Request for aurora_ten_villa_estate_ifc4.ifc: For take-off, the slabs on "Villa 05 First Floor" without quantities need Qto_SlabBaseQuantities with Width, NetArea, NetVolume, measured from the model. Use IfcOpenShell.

First a look at what the model holds.

```python
import ifcopenshell
import ifcopenshell.util.element
import ifcopenshell.util.unit

model = ifcopenshell.open("aurora_ten_villa_estate_ifc4.ifc")
print(model.schema)
for unit_type in ("LENGTHUNIT", "AREAUNIT", "VOLUMEUNIT"):
    print(unit_type, ifcopenshell.util.unit.calculate_unit_scale(model, unit_type))
storey = next(s for s in model.by_type("IfcBuildingStorey") if s.Name == "Villa 05 First Floor")
slabs = [e for e in ifcopenshell.util.element.get_decomposition(storey) if e.is_a("IfcSlab")]
for e in sorted(slabs, key=lambda e: e.id()):
    print(e.id(), e.is_a(), e.Name, list(ifcopenshell.util.element.get_psets(e, qtos_only=True)), sep=" | ")
```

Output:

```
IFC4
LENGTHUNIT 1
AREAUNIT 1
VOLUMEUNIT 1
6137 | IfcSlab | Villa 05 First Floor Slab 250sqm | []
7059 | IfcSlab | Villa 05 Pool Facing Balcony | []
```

```python
import ifcopenshell
import ifcopenshell.api.pset
import ifcopenshell.geom
import ifcopenshell.util.element
import ifcopenshell.util.shape
import ifcopenshell.util.unit

model = ifcopenshell.open("aurora_ten_villa_estate_ifc4.ifc")
unit_scale = ifcopenshell.util.unit.calculate_unit_scale(model)
area_scale = ifcopenshell.util.unit.calculate_unit_scale(model, "AREAUNIT")
volume_scale = ifcopenshell.util.unit.calculate_unit_scale(model, "VOLUMEUNIT")
settings = ifcopenshell.geom.settings()

storey = next(s for s in model.by_type("IfcBuildingStorey") if s.Name == "Villa 05 First Floor")
slabs = [e for e in ifcopenshell.util.element.get_decomposition(storey) if e.is_a("IfcSlab")]

for e in sorted(slabs, key=lambda e: e.id()):
    if ifcopenshell.util.element.get_psets(e, qtos_only=True, should_inherit=False):
        continue
    # Geometry comes back in metres, in the element's own axes.
    shape = ifcopenshell.geom.create_shape(settings, e)
    values = {
        "Width": ifcopenshell.util.shape.get_z(shape.geometry) / unit_scale,
        "NetArea": ifcopenshell.util.shape.get_footprint_area(shape.geometry) / area_scale,
        "NetVolume": ifcopenshell.util.shape.get_volume(shape.geometry) / volume_scale,
    }
    qto = ifcopenshell.api.pset.add_qto(model, product=e, name="Qto_SlabBaseQuantities")
    ifcopenshell.api.pset.edit_qto(model, qto=qto, properties=values)
    print(e.id(), {k: round(v, 3) for k, v in values.items()})

model.write("aurora_ten_villa_estate_ifc4_edited.ifc")
```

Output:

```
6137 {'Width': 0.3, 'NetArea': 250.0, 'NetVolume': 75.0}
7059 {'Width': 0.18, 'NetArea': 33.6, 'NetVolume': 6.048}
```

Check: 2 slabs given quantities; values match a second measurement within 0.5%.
